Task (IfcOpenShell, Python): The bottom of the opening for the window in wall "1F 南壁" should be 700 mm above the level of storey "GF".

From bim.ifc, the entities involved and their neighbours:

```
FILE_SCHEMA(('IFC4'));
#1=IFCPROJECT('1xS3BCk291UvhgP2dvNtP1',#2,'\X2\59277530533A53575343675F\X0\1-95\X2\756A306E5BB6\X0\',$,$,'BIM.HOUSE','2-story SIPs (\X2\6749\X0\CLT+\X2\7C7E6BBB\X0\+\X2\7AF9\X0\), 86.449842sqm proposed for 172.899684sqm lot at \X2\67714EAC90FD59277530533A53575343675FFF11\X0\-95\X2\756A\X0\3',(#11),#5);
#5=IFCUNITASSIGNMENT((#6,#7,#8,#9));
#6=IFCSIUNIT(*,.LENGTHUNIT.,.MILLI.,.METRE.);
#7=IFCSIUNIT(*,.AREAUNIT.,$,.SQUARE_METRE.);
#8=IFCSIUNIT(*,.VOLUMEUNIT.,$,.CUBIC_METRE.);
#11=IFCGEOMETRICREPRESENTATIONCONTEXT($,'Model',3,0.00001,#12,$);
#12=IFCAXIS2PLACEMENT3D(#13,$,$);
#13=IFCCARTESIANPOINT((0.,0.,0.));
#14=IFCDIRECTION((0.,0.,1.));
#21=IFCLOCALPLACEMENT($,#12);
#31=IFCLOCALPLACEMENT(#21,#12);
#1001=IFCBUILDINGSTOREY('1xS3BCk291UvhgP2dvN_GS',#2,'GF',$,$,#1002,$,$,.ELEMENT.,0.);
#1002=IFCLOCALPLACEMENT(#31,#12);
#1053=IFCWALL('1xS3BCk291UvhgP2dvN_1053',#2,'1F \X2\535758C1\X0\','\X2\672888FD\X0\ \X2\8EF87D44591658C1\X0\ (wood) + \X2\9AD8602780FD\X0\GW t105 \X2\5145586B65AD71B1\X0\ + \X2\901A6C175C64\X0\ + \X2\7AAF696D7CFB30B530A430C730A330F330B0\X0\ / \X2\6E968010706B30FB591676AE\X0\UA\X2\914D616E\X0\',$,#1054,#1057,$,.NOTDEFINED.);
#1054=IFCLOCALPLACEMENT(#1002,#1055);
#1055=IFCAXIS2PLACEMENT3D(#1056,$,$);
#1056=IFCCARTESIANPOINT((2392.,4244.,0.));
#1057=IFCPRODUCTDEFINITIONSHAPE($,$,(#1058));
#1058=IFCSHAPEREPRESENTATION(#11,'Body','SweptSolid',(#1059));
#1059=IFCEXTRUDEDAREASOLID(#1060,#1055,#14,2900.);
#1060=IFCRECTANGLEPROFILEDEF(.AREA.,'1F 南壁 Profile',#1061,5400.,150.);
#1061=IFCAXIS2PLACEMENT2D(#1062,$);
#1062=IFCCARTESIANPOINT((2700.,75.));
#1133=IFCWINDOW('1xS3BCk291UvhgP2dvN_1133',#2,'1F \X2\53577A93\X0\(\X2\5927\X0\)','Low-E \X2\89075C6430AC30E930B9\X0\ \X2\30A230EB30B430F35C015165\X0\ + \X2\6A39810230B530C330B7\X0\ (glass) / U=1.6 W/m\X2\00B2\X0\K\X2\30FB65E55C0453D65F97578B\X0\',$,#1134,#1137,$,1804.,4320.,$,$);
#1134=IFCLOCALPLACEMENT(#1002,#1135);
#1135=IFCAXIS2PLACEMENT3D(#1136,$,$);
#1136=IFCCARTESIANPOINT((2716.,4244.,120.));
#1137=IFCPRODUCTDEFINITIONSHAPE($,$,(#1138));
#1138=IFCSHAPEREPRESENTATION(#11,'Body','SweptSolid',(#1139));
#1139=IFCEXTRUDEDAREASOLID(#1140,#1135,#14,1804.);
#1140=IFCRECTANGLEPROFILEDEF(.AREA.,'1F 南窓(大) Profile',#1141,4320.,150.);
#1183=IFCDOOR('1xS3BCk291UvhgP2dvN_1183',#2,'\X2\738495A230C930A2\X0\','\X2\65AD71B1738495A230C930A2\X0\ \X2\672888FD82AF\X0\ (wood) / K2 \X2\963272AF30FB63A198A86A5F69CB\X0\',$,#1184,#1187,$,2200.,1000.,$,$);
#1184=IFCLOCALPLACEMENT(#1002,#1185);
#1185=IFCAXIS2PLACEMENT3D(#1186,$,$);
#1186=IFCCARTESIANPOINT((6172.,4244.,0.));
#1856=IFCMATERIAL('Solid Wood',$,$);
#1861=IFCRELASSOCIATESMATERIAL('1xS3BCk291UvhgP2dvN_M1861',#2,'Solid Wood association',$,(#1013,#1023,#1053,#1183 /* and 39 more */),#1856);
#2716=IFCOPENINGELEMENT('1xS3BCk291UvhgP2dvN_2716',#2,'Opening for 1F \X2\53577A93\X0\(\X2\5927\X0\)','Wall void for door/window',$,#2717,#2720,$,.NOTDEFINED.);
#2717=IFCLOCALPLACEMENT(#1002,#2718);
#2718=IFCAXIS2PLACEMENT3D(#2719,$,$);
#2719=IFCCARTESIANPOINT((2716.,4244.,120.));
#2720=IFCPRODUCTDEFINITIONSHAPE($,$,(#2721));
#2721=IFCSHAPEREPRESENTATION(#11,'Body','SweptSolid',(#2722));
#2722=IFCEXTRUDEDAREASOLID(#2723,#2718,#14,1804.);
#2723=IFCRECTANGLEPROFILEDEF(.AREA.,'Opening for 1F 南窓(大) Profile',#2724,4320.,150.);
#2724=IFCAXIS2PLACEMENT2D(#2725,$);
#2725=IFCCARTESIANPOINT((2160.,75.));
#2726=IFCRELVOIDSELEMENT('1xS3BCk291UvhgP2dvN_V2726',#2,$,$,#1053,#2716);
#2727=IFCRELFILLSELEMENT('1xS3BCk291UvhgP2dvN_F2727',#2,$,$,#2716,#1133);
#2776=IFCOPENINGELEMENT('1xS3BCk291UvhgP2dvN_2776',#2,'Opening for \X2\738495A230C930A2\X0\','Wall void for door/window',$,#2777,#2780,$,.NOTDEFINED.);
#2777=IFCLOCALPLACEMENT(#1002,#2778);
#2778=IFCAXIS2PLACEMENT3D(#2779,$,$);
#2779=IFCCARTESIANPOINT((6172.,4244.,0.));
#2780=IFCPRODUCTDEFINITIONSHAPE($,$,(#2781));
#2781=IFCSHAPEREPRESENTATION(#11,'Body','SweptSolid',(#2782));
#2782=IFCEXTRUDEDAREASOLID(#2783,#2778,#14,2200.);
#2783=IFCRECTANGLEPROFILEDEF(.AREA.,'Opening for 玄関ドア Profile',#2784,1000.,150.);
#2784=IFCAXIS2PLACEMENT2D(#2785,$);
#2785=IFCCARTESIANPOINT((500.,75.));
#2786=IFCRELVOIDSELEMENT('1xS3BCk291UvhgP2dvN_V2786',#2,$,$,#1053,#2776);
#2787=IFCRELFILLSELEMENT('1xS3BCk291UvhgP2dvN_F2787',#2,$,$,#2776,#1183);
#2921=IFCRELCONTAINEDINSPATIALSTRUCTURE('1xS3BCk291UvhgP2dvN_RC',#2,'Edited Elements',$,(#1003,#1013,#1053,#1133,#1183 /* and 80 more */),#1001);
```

```python
import numpy as np
import ifcopenshell
import ifcopenshell.api.geometry
import ifcopenshell.geom
import ifcopenshell.util.element
import ifcopenshell.util.placement
import ifcopenshell.util.shape
import ifcopenshell.util.unit

model = ifcopenshell.open("bim.ifc")
unit_scale = ifcopenshell.util.unit.calculate_unit_scale(model)

window = model.by_id(1133)
opening = window.FillsVoids[0].RelatingOpeningElement
storey = ifcopenshell.util.element.get_container(window, ifc_class="IfcBuildingStorey")
level = ifcopenshell.util.placement.get_local_placement(storey.ObjectPlacement)[2, 3]

# The opening's origin need not be at the sill, so measure its lowest point.
shape = ifcopenshell.geom.create_shape(ifcopenshell.geom.settings(), opening)
bottom = ifcopenshell.util.shape.get_shape_bottom_elevation(shape, shape.geometry) / unit_scale
dz = level + 700.0 - bottom

shift = np.array([0.0, 0.0, dz])
# The window is not placed relative to its opening, so move both.
for product in (opening, window):
    matrix = ifcopenshell.util.placement.get_local_placement(product.ObjectPlacement)
    matrix[:3, 3] += shift
    ifcopenshell.api.geometry.edit_object_placement(model, product=product, matrix=matrix, is_si=False)

print(f"moved by {dz * unit_scale:+.3f} m")

model.write("bim-out.ifc")
```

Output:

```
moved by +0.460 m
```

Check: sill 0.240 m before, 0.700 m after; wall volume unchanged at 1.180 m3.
